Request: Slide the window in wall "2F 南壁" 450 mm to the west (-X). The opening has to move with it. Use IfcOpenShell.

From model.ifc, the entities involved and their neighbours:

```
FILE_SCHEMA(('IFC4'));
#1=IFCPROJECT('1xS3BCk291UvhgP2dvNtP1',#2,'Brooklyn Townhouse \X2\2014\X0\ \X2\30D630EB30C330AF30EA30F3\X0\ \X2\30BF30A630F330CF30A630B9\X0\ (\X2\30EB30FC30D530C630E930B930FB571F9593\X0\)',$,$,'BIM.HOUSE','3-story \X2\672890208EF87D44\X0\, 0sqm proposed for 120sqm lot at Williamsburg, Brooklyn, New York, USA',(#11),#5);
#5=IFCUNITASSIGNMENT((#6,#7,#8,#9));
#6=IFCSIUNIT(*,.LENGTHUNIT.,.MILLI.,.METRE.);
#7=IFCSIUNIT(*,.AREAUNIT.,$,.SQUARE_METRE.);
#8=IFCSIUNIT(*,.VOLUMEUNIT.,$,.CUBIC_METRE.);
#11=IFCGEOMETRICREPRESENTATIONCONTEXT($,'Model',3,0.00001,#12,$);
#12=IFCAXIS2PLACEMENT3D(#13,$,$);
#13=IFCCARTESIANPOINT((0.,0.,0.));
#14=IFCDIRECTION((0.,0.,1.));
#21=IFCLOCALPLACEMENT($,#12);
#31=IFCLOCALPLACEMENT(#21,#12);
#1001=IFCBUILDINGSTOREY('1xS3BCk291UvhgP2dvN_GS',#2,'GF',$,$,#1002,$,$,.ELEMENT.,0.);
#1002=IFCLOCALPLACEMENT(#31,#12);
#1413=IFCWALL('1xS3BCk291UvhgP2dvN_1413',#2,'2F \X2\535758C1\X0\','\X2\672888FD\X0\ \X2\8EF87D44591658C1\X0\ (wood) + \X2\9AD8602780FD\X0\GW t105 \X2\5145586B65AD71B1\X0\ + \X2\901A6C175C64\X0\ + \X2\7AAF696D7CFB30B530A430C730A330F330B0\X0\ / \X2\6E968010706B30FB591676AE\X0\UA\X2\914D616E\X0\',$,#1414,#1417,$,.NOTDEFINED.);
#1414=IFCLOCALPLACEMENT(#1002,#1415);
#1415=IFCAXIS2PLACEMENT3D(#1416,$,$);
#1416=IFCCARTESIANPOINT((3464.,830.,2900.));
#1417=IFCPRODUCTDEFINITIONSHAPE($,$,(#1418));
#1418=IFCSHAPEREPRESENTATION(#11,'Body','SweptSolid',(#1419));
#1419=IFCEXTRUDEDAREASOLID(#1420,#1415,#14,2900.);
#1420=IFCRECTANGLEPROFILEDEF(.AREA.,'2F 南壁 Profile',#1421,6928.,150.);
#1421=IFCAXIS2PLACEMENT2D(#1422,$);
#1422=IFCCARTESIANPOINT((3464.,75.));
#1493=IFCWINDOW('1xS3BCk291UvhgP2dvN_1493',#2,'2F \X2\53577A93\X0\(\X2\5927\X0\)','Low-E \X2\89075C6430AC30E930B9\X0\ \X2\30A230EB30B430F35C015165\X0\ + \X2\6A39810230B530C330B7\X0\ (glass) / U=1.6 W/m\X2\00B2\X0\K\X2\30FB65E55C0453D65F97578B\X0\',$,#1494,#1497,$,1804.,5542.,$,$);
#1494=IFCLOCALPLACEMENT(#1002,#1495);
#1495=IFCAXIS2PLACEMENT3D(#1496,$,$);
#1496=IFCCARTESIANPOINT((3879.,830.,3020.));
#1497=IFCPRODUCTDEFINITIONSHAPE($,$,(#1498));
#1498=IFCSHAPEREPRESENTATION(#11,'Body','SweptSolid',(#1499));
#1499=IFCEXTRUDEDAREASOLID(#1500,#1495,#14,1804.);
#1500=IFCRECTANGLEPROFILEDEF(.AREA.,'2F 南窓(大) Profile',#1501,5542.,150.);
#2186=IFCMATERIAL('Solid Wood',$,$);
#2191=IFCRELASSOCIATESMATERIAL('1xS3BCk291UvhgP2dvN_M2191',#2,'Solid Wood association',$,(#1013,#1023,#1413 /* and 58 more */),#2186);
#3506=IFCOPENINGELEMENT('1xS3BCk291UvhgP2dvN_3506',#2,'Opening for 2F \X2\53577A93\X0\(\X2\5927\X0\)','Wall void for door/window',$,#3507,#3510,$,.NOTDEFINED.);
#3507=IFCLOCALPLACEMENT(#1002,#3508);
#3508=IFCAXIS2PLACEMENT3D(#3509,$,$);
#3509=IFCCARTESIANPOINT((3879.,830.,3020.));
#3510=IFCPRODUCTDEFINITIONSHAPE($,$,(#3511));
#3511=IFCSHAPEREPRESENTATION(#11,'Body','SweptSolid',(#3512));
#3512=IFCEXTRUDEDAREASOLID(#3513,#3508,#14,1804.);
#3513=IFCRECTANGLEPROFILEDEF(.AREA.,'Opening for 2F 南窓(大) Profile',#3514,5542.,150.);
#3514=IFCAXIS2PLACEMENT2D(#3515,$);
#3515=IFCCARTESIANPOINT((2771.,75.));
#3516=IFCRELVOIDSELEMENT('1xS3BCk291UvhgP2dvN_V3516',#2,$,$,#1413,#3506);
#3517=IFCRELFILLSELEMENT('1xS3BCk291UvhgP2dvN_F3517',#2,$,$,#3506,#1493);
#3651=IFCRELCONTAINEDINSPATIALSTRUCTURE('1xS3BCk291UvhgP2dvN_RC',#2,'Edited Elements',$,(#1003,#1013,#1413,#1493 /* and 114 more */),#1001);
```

```python
import ifcopenshell
import ifcopenshell.api.geometry
import ifcopenshell.util.placement
import ifcopenshell.util.unit

model = ifcopenshell.open("model.ifc")
unit_scale = ifcopenshell.util.unit.calculate_unit_scale(model)

window = model.by_guid("1xS3BCk291UvhgP2dvN_1493")
opening = window.FillsVoids[0].RelatingOpeningElement
wall = opening.VoidsElements[0].RelatingBuildingElement

wall_matrix = ifcopenshell.util.placement.get_local_placement(wall.ObjectPlacement)
shift = wall_matrix[:3, 0] * -0.45 / unit_scale
before = ifcopenshell.util.placement.get_local_placement(window.ObjectPlacement)[:3, 3].copy()

# The window is not placed relative to its opening, so move both.
for product in (opening, window):
    matrix = ifcopenshell.util.placement.get_local_placement(product.ObjectPlacement)
    matrix[:3, 3] += shift
    ifcopenshell.api.geometry.edit_object_placement(model, product=product, matrix=matrix, is_si=False)

after = ifcopenshell.util.placement.get_local_placement(window.ObjectPlacement)[:3, 3]
print("window moved by", (after - before).round(3) + 0.0)

model.write("model_edited.ifc")
```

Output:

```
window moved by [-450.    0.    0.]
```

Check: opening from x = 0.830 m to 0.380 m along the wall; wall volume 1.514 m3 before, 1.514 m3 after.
